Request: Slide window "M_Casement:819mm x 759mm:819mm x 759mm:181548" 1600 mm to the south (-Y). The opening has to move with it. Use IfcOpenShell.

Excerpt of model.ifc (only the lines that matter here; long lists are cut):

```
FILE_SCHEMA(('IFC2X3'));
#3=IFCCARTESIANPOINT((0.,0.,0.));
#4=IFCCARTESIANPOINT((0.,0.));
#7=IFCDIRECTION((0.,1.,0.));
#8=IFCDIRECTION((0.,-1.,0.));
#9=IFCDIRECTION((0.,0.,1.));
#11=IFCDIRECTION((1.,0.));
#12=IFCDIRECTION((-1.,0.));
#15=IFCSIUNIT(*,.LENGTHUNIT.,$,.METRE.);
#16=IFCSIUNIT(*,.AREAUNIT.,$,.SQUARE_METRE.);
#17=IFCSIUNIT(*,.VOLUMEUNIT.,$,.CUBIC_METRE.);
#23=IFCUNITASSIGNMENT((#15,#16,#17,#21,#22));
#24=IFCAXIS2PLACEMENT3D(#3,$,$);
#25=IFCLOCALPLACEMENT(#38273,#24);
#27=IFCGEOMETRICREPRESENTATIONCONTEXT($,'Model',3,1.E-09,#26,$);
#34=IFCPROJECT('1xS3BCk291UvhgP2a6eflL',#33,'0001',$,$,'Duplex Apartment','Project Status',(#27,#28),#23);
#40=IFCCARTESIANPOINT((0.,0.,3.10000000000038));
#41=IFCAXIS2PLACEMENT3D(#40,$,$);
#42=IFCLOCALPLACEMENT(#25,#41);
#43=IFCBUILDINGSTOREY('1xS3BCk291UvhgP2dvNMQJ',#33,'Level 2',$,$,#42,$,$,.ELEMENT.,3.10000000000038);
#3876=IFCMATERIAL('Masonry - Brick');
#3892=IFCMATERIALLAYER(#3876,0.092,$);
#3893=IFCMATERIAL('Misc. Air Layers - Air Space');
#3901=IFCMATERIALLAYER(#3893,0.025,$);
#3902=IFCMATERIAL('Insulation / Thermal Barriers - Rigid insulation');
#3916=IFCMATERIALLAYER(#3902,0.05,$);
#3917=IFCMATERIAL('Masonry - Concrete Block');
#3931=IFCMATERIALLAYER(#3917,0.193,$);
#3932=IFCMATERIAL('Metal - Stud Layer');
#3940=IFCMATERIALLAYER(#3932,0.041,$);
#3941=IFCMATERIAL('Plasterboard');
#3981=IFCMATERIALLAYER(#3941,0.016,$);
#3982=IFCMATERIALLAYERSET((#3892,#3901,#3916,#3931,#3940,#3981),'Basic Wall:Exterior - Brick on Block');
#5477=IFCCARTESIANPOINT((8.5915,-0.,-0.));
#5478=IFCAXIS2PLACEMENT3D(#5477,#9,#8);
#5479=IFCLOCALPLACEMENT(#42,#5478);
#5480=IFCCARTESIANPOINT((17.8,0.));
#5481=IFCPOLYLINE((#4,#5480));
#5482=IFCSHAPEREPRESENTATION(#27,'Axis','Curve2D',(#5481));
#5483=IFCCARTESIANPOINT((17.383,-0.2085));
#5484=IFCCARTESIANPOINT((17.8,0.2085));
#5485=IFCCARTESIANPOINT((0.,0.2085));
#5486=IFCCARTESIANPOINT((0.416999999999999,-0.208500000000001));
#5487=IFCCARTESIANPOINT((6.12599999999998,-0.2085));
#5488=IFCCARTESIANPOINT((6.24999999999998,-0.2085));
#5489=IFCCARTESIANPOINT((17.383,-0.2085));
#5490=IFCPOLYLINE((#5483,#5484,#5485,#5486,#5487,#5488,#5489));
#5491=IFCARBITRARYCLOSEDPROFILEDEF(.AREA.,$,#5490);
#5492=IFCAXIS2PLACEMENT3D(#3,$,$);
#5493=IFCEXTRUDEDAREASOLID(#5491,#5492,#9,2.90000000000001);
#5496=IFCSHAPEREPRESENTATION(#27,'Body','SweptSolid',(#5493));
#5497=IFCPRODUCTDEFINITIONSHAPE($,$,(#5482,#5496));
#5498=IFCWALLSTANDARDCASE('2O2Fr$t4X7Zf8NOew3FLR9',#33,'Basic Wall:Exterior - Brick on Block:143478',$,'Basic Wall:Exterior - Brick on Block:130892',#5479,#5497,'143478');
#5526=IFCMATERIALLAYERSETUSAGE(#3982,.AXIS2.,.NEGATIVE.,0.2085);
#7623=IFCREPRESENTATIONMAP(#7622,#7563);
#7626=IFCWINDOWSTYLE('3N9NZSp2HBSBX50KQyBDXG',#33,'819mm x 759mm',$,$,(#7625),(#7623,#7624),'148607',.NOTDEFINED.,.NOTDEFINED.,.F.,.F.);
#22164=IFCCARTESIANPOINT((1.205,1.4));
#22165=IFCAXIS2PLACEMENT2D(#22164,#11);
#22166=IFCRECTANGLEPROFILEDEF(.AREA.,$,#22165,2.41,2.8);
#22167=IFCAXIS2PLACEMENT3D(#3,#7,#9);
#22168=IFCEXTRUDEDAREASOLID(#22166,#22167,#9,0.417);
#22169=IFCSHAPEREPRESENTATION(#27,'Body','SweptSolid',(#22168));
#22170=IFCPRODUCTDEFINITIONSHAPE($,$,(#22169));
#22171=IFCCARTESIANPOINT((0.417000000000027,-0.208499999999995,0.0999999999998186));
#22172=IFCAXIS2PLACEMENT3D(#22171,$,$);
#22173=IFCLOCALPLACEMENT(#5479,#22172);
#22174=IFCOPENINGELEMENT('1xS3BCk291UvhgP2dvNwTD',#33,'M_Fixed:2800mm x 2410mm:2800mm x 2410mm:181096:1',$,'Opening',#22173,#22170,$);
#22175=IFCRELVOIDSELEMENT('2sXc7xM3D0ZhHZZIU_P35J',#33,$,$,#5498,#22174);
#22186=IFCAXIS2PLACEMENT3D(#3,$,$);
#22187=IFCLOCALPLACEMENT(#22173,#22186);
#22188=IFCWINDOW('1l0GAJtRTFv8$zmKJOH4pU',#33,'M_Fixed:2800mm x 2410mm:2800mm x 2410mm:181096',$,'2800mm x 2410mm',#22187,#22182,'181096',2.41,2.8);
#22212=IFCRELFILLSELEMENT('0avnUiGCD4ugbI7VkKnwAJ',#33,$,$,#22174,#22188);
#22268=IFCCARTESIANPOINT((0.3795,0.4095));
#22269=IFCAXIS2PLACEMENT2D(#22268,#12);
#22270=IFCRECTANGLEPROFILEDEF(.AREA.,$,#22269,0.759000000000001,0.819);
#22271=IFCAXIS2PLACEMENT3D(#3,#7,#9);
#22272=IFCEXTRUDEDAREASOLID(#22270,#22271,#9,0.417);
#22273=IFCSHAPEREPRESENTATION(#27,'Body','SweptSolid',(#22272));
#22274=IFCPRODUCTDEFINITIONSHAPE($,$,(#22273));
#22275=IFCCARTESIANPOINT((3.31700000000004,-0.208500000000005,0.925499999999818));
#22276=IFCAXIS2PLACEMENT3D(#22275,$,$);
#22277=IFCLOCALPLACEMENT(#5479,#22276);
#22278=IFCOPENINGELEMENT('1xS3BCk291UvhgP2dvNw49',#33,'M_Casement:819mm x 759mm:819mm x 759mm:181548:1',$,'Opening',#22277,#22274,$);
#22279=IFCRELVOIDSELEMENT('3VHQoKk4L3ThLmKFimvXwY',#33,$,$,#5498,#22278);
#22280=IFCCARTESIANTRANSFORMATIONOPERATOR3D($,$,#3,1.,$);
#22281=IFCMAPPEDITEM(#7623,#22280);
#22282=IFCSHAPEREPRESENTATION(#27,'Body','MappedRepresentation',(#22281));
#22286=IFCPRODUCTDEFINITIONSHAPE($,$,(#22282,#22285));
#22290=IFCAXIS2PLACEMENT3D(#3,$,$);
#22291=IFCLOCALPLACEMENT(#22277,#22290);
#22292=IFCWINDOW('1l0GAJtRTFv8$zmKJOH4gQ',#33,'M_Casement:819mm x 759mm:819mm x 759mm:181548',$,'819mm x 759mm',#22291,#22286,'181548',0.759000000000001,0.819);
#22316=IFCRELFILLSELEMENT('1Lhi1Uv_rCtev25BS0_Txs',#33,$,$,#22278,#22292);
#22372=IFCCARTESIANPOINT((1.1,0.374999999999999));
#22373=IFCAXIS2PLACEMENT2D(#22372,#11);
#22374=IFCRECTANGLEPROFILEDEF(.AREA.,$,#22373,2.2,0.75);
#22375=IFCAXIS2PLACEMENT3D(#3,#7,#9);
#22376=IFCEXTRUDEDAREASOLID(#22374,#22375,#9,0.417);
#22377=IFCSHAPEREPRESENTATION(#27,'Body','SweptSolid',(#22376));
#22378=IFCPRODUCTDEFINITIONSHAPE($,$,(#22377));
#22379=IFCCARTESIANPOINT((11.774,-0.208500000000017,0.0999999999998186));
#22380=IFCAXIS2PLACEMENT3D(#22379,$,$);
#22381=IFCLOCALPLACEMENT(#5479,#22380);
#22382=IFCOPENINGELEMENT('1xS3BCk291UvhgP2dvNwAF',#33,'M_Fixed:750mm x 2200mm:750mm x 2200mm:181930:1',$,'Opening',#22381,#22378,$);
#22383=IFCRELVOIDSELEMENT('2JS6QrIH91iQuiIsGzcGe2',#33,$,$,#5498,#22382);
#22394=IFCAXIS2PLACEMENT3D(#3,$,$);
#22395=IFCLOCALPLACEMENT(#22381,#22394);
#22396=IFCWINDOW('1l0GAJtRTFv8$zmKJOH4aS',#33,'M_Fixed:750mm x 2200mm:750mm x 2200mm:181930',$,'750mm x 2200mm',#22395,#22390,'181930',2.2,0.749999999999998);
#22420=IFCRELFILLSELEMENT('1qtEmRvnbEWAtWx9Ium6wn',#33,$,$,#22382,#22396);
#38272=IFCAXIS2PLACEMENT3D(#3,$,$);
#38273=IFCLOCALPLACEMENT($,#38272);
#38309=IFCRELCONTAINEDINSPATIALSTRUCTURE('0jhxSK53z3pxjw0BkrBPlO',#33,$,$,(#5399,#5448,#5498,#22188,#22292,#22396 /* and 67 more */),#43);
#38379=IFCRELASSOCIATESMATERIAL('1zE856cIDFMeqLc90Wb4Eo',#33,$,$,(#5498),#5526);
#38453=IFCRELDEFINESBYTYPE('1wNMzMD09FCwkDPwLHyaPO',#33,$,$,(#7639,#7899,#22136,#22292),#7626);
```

```python
import ifcopenshell
import ifcopenshell.api.geometry
import ifcopenshell.util.placement

model = ifcopenshell.open("model.ifc")

window = model.by_id(22292)
opening = window.FillsVoids[0].RelatingOpeningElement
wall = opening.VoidsElements[0].RelatingBuildingElement

wall_matrix = ifcopenshell.util.placement.get_local_placement(wall.ObjectPlacement)
shift = wall_matrix[:3, 0] * 1.6
before = ifcopenshell.util.placement.get_local_placement(window.ObjectPlacement)[:3, 3].copy()

# The window is placed relative to its opening, so it follows when the opening moves.
matrix = ifcopenshell.util.placement.get_local_placement(opening.ObjectPlacement)
matrix[:3, 3] += shift
ifcopenshell.api.geometry.edit_object_placement(
    model, product=opening, matrix=matrix, is_si=False, should_transform_children=True
)

after = ifcopenshell.util.placement.get_local_placement(window.ObjectPlacement)[:3, 3]
print("window moved by", (after - before).round(3) + 0.0)

model.write("model_updated.ifc")
```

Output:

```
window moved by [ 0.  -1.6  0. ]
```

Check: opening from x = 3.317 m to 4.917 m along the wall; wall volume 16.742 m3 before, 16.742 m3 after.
